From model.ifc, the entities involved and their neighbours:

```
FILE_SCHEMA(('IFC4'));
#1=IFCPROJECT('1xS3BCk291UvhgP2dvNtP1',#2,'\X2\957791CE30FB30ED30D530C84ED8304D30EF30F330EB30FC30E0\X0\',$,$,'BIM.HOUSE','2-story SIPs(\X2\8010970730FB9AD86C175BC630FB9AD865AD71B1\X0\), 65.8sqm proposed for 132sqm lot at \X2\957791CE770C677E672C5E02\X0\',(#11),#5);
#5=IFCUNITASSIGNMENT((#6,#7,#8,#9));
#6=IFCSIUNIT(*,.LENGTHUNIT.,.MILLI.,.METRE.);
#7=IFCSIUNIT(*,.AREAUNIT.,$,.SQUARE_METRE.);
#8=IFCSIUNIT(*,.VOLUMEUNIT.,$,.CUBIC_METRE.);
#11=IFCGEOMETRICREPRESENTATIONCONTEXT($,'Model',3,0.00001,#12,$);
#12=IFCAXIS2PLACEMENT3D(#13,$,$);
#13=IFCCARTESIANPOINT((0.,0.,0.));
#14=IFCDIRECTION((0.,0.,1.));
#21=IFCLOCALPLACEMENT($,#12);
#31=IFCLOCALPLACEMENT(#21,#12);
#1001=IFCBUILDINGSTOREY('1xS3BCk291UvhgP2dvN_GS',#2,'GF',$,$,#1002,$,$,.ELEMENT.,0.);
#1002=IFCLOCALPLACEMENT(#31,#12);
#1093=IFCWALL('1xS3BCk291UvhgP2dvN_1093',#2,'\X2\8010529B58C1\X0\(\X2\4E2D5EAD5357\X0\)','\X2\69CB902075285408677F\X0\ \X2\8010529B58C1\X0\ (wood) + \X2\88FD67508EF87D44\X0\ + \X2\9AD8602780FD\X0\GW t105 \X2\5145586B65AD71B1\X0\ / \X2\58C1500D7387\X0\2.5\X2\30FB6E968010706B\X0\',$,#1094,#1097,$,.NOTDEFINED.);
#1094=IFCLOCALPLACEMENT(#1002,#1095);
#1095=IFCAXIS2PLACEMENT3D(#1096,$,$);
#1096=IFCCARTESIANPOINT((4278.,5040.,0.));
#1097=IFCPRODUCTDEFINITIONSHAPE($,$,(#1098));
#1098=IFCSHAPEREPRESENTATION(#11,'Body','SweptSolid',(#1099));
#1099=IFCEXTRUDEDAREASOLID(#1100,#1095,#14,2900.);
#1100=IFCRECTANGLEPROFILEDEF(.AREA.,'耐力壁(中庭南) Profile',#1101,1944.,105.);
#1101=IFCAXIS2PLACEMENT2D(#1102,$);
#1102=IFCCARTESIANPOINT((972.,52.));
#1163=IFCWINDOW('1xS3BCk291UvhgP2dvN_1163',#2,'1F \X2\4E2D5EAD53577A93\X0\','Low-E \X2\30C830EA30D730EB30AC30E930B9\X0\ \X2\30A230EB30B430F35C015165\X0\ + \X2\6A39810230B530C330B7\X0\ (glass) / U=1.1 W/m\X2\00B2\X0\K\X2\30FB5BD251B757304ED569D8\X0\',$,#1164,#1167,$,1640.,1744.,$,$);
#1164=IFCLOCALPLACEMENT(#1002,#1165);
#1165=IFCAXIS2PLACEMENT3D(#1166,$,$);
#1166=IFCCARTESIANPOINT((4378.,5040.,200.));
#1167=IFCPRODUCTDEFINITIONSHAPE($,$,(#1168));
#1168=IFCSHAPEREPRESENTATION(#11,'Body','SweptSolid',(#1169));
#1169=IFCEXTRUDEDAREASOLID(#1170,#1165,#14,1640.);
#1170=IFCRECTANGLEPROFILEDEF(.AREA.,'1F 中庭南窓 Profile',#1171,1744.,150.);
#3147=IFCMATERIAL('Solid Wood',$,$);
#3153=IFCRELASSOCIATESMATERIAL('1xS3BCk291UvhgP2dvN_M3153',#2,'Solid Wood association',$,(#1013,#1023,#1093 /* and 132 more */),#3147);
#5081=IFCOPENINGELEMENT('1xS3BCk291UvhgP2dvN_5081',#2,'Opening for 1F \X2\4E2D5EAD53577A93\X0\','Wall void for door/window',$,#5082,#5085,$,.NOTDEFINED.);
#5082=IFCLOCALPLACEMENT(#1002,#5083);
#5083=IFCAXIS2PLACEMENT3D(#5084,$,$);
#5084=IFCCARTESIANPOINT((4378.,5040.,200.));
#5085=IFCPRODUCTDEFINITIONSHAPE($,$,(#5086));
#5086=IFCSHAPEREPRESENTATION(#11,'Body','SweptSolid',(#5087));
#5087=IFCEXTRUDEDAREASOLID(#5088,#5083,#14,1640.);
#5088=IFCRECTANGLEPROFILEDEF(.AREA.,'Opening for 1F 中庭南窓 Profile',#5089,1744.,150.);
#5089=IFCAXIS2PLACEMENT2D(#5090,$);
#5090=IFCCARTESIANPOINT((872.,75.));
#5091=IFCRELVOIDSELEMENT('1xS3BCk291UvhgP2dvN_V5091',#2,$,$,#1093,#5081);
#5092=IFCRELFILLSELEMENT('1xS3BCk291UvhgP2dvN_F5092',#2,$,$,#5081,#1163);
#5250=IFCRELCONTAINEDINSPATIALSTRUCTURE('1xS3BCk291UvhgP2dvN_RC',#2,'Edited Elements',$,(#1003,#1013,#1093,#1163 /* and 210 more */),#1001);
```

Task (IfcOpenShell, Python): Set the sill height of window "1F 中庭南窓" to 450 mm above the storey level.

```python
import numpy as np
import ifcopenshell
import ifcopenshell.api.geometry
import ifcopenshell.geom
import ifcopenshell.util.element
import ifcopenshell.util.placement
import ifcopenshell.util.shape
import ifcopenshell.util.unit

model = ifcopenshell.open("model.ifc")
unit_scale = ifcopenshell.util.unit.calculate_unit_scale(model)

window = model.by_guid("1xS3BCk291UvhgP2dvN_1163")
opening = window.FillsVoids[0].RelatingOpeningElement
storey = ifcopenshell.util.element.get_container(window, ifc_class="IfcBuildingStorey")
level = ifcopenshell.util.placement.get_local_placement(storey.ObjectPlacement)[2, 3]

# The opening's origin need not be at the sill, so measure its lowest point.
shape = ifcopenshell.geom.create_shape(ifcopenshell.geom.settings(), opening)
bottom = ifcopenshell.util.shape.get_shape_bottom_elevation(shape, shape.geometry) / unit_scale
dz = level + 0.45 / unit_scale - bottom

shift = np.array([0.0, 0.0, dz])
# The window is not placed relative to its opening, so move both.
for product in (opening, window):
    matrix = ifcopenshell.util.placement.get_local_placement(product.ObjectPlacement)
    matrix[:3, 3] += shift
    ifcopenshell.api.geometry.edit_object_placement(model, product=product, matrix=matrix, is_si=False)

print(f"moved by {dz * unit_scale:+.3f} m")

model.write("model_edited.ifc")
```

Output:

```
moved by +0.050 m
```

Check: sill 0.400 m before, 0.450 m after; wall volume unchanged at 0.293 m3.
